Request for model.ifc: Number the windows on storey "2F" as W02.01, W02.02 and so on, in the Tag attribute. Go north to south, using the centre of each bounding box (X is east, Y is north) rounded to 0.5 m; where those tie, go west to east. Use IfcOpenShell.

First a look at what the model holds.

```python
import ifcopenshell
import ifcopenshell.util.element
import ifcopenshell.util.placement

model = ifcopenshell.open("model.ifc")
print(model.schema)
storey = next(s for s in model.by_type("IfcBuildingStorey") if s.Name == "2F")
windows = [e for e in ifcopenshell.util.element.get_decomposition(storey) if e.is_a("IfcWindow")]
for e in sorted(windows, key=lambda e: e.id()):
    origin = ifcopenshell.util.placement.get_local_placement(e.ObjectPlacement)[:3, 3]
    print(e.id(), e.Tag, e.Name, origin.round(2) + 0.0, sep=" | ")
```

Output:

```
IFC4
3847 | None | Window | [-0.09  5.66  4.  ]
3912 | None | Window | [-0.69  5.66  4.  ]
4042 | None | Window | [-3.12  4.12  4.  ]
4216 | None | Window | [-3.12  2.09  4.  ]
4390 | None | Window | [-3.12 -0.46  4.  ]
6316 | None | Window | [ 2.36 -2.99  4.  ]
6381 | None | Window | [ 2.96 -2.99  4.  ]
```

```python
import ifcopenshell
import ifcopenshell.geom
import ifcopenshell.util.element
import ifcopenshell.util.shape

model = ifcopenshell.open("model.ifc")
settings = ifcopenshell.geom.settings()
settings.set("use-world-coords", True)


def centre(element):
    shape = ifcopenshell.geom.create_shape(settings, element)
    return ifcopenshell.util.shape.get_bbox_centroid(shape.geometry)


storey = next(s for s in model.by_type("IfcBuildingStorey") if s.Name == "2F")
windows = [e for e in ifcopenshell.util.element.get_decomposition(storey) if e.is_a("IfcWindow")]

# Insertion points can sit at a corner or the storey origin, so sort by the geometry (in metres).
centres = {e: centre(e) for e in windows}
windows.sort(key=lambda e: (-round(centres[e][1] / 0.5), centres[e][0]))

for i, e in enumerate(windows, start=1):
    number = f"W02.{i:02d}"
    e.Tag = number
    print(e.id(), number)

model.write("model_updated.ifc")
```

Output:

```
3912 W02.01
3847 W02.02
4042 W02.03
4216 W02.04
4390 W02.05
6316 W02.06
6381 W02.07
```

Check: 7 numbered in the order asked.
